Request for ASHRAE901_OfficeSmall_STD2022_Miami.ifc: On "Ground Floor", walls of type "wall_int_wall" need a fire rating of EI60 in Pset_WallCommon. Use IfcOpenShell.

First a look at what the model holds.

```python
import ifcopenshell
import ifcopenshell.util.element

model = ifcopenshell.open("ASHRAE901_OfficeSmall_STD2022_Miami.ifc")
print(model.schema)
storey = next(s for s in model.by_type("IfcBuildingStorey") if s.Name == "Ground Floor")
walls = [e for e in ifcopenshell.util.element.get_decomposition(storey) if e.is_a("IfcWall")]
seen = {}
for e in walls:
    element_type = ifcopenshell.util.element.get_type(e)
    key = (element_type.Name if element_type != e and element_type else None, ifcopenshell.util.element.get_pset(e, "Pset_WallCommon", "FireRating"))
    seen[key] = seen.get(key, 0) + 1
for (name, value), count in sorted(seen.items(), key=str):
    print(count, "x", name, "|", value)
```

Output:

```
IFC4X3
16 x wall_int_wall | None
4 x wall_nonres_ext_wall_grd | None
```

```python
import ifcopenshell
import ifcopenshell.api.pset
import ifcopenshell.util.element

model = ifcopenshell.open("ASHRAE901_OfficeSmall_STD2022_Miami.ifc")

storey = next(s for s in model.by_type("IfcBuildingStorey") if s.Name == "Ground Floor")
walls = [e for e in ifcopenshell.util.element.get_decomposition(storey) if e.is_a("IfcWall")]

count = 0
for e in walls:
    element_type = ifcopenshell.util.element.get_type(e)
    if element_type in (None, e) or element_type.Name != "wall_int_wall":
        continue
    # add_pset returns the element's existing set when there is one.
    pset = ifcopenshell.api.pset.add_pset(model, product=e, name="Pset_WallCommon")
    ifcopenshell.api.pset.edit_pset(model, pset=pset, properties={"FireRating": "EI60"})
    count += 1

print(count, "walls updated")

model.write("ASHRAE901_OfficeSmall_STD2022_Miami_updated.ifc")
```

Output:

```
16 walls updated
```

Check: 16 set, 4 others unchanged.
